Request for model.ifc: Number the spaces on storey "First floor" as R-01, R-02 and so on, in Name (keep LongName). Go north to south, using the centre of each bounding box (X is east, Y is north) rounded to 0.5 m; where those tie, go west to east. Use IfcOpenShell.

First a look at what the model holds.

```python
import ifcopenshell
import ifcopenshell.util.element
import ifcopenshell.util.placement

model = ifcopenshell.open("model.ifc")
print(model.schema)
storey = next(s for s in model.by_type("IfcBuildingStorey") if s.Name == "First floor")
spaces = [e for e in ifcopenshell.util.element.get_decomposition(storey) if e.is_a("IfcSpace")]
for e in sorted(spaces, key=lambda e: e.id()):
    origin = ifcopenshell.util.placement.get_local_placement(e.ObjectPlacement)[:3, 3]
    print(e.id(), e.Name, e.LongName, origin.round(2) + 0.0, sep=" | ")
```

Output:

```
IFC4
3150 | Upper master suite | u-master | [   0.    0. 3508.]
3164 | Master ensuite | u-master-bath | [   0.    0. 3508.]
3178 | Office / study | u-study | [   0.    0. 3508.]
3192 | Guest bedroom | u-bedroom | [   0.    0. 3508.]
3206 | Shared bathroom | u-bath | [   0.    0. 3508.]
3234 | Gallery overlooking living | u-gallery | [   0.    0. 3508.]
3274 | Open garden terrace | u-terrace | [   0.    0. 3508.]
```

```python
import ifcopenshell
import ifcopenshell.geom
import ifcopenshell.util.element
import ifcopenshell.util.shape

model = ifcopenshell.open("model.ifc")
settings = ifcopenshell.geom.settings()
settings.set("use-world-coords", True)


def centre(element):
    shape = ifcopenshell.geom.create_shape(settings, element)
    return ifcopenshell.util.shape.get_bbox_centroid(shape.geometry)


storey = next(s for s in model.by_type("IfcBuildingStorey") if s.Name == "First floor")
spaces = [e for e in ifcopenshell.util.element.get_decomposition(storey) if e.is_a("IfcSpace")]

# Insertion points can sit at a corner or the storey origin, so sort by the geometry (in metres).
centres = {e: centre(e) for e in spaces}
spaces.sort(key=lambda e: (-round(centres[e][1] / 0.5), centres[e][0]))

for i, e in enumerate(spaces, start=1):
    number = f"R-{i:02d}"
    e.Name = number
    print(e.id(), number)

model.write("model_updated.ifc")
```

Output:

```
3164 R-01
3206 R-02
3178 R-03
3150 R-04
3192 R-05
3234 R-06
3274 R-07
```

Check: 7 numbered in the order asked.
